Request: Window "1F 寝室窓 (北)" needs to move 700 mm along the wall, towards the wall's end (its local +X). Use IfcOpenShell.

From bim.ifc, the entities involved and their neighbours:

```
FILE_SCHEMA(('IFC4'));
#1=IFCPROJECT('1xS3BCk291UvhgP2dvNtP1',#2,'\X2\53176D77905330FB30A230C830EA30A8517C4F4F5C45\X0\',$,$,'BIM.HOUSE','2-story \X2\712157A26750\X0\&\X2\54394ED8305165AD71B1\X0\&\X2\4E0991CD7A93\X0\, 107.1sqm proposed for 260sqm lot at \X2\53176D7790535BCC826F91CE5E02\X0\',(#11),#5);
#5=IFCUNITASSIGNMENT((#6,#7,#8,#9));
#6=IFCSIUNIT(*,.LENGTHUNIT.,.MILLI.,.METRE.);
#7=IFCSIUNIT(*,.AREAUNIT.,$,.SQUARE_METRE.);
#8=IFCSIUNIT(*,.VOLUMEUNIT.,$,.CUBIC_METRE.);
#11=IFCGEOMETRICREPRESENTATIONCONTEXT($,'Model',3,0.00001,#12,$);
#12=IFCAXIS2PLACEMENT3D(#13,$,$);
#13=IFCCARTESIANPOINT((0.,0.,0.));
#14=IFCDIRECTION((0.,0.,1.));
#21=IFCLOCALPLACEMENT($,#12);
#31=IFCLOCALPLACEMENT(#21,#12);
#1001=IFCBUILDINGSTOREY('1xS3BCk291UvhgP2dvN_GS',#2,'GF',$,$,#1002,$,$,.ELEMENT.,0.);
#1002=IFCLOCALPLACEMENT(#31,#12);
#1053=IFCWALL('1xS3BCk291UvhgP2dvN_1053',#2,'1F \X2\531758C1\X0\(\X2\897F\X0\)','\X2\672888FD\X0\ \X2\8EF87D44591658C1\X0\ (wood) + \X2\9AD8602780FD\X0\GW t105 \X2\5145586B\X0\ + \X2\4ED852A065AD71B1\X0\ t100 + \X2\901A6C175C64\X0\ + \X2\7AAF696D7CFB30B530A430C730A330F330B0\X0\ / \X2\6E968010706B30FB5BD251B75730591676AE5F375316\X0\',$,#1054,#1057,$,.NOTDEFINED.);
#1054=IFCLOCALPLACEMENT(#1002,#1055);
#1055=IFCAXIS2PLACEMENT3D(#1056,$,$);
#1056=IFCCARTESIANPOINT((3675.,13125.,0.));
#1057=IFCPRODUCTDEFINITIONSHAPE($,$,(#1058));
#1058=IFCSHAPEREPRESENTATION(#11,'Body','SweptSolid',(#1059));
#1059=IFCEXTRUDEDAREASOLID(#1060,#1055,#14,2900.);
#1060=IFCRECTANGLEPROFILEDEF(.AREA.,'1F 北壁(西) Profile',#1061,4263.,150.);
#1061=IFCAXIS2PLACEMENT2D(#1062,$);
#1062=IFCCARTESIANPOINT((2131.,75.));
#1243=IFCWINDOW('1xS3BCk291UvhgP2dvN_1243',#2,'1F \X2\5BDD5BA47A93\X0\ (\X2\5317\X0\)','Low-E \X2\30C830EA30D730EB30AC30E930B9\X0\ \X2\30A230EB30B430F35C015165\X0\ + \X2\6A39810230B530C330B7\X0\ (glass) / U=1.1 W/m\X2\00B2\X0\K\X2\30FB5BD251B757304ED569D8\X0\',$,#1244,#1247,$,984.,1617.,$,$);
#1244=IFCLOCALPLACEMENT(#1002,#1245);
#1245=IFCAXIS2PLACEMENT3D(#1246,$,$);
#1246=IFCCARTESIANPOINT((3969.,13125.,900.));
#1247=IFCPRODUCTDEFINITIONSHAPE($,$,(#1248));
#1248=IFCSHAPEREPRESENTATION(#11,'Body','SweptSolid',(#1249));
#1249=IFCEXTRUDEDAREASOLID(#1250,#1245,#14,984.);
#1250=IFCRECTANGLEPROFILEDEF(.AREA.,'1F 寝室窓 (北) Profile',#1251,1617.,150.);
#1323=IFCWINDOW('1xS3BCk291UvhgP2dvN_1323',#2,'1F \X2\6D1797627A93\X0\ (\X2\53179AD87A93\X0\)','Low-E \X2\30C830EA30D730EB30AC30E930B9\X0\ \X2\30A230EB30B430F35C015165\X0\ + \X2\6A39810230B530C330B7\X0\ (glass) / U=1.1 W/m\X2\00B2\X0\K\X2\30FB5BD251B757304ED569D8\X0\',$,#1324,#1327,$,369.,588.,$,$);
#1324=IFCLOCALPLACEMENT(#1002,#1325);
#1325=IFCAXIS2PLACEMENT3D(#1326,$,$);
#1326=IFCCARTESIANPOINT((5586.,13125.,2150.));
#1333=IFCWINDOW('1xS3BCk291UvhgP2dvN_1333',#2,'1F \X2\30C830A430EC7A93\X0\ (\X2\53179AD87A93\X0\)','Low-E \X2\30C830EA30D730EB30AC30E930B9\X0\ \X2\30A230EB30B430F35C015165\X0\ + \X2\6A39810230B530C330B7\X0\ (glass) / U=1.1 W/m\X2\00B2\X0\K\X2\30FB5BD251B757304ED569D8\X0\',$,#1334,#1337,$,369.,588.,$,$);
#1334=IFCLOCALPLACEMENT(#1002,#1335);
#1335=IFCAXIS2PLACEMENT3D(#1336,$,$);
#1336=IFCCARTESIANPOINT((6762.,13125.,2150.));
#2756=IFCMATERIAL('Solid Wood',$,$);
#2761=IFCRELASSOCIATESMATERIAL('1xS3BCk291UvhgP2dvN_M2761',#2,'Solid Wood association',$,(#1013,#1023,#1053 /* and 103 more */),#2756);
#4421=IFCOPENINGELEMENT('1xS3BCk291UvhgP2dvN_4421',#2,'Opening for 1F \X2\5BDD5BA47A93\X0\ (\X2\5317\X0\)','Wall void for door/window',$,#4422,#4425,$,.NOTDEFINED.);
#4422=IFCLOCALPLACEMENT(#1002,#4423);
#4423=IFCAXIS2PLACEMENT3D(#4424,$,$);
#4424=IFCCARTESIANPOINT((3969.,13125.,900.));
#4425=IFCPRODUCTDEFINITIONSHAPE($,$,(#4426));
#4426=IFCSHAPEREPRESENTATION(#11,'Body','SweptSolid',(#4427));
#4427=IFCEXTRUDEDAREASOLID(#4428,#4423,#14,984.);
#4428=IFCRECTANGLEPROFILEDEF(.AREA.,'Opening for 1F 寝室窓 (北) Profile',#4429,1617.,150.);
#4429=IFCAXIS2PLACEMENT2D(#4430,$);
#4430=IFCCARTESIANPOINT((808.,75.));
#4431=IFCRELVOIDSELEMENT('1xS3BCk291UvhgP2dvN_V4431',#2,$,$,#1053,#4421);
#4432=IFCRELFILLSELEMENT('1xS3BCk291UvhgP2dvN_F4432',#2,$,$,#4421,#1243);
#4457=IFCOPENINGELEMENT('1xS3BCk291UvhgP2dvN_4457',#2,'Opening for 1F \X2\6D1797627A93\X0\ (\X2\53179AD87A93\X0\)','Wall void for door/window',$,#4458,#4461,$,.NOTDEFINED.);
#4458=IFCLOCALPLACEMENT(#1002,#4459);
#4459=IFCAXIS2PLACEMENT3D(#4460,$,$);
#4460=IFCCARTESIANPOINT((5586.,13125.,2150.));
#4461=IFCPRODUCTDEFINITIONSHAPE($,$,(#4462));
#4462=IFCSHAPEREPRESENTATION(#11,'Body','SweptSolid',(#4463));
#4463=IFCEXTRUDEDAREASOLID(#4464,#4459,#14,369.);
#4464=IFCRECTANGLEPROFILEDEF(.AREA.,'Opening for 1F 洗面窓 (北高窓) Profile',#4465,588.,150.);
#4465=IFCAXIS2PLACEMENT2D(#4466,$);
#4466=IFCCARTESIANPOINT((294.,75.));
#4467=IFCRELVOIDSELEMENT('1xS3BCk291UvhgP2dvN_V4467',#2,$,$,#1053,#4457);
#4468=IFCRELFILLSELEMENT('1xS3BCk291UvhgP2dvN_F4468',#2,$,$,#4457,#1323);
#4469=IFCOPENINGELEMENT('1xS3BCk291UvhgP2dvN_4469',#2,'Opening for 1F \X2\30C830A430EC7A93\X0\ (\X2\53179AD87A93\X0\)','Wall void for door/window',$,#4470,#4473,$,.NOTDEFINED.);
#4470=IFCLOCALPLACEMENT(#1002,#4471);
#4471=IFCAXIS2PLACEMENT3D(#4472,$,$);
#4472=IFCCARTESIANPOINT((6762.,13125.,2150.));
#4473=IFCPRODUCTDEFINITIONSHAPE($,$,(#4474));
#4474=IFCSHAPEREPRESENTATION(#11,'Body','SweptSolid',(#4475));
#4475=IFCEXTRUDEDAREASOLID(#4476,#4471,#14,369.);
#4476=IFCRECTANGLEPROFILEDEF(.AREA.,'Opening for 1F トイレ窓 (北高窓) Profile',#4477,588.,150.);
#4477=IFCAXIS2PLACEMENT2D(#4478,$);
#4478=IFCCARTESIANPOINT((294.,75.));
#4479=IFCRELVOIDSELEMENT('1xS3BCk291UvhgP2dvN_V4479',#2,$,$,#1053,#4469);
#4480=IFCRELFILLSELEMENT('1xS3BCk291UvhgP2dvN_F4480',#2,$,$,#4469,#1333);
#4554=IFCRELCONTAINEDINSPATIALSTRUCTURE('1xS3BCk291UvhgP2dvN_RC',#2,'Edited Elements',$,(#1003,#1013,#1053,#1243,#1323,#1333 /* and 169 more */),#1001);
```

```python
import ifcopenshell
import ifcopenshell.api.geometry
import ifcopenshell.util.placement
import ifcopenshell.util.unit

model = ifcopenshell.open("bim.ifc")
unit_scale = ifcopenshell.util.unit.calculate_unit_scale(model)

window = model.by_guid("1xS3BCk291UvhgP2dvN_1243")
opening = window.FillsVoids[0].RelatingOpeningElement
wall = opening.VoidsElements[0].RelatingBuildingElement

wall_matrix = ifcopenshell.util.placement.get_local_placement(wall.ObjectPlacement)
shift = wall_matrix[:3, 0] * 0.7 / unit_scale
before = ifcopenshell.util.placement.get_local_placement(window.ObjectPlacement)[:3, 3].copy()

# The window is not placed relative to its opening, so move both.
for product in (opening, window):
    matrix = ifcopenshell.util.placement.get_local_placement(product.ObjectPlacement)
    matrix[:3, 3] += shift
    ifcopenshell.api.geometry.edit_object_placement(model, product=product, matrix=matrix, is_si=False)

after = ifcopenshell.util.placement.get_local_placement(window.ObjectPlacement)[:3, 3]
print("window moved by", (after - before).round(3) + 0.0)

model.write("bim_rev.ifc")
```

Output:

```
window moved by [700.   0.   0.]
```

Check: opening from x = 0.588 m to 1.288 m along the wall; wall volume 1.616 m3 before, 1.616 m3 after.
